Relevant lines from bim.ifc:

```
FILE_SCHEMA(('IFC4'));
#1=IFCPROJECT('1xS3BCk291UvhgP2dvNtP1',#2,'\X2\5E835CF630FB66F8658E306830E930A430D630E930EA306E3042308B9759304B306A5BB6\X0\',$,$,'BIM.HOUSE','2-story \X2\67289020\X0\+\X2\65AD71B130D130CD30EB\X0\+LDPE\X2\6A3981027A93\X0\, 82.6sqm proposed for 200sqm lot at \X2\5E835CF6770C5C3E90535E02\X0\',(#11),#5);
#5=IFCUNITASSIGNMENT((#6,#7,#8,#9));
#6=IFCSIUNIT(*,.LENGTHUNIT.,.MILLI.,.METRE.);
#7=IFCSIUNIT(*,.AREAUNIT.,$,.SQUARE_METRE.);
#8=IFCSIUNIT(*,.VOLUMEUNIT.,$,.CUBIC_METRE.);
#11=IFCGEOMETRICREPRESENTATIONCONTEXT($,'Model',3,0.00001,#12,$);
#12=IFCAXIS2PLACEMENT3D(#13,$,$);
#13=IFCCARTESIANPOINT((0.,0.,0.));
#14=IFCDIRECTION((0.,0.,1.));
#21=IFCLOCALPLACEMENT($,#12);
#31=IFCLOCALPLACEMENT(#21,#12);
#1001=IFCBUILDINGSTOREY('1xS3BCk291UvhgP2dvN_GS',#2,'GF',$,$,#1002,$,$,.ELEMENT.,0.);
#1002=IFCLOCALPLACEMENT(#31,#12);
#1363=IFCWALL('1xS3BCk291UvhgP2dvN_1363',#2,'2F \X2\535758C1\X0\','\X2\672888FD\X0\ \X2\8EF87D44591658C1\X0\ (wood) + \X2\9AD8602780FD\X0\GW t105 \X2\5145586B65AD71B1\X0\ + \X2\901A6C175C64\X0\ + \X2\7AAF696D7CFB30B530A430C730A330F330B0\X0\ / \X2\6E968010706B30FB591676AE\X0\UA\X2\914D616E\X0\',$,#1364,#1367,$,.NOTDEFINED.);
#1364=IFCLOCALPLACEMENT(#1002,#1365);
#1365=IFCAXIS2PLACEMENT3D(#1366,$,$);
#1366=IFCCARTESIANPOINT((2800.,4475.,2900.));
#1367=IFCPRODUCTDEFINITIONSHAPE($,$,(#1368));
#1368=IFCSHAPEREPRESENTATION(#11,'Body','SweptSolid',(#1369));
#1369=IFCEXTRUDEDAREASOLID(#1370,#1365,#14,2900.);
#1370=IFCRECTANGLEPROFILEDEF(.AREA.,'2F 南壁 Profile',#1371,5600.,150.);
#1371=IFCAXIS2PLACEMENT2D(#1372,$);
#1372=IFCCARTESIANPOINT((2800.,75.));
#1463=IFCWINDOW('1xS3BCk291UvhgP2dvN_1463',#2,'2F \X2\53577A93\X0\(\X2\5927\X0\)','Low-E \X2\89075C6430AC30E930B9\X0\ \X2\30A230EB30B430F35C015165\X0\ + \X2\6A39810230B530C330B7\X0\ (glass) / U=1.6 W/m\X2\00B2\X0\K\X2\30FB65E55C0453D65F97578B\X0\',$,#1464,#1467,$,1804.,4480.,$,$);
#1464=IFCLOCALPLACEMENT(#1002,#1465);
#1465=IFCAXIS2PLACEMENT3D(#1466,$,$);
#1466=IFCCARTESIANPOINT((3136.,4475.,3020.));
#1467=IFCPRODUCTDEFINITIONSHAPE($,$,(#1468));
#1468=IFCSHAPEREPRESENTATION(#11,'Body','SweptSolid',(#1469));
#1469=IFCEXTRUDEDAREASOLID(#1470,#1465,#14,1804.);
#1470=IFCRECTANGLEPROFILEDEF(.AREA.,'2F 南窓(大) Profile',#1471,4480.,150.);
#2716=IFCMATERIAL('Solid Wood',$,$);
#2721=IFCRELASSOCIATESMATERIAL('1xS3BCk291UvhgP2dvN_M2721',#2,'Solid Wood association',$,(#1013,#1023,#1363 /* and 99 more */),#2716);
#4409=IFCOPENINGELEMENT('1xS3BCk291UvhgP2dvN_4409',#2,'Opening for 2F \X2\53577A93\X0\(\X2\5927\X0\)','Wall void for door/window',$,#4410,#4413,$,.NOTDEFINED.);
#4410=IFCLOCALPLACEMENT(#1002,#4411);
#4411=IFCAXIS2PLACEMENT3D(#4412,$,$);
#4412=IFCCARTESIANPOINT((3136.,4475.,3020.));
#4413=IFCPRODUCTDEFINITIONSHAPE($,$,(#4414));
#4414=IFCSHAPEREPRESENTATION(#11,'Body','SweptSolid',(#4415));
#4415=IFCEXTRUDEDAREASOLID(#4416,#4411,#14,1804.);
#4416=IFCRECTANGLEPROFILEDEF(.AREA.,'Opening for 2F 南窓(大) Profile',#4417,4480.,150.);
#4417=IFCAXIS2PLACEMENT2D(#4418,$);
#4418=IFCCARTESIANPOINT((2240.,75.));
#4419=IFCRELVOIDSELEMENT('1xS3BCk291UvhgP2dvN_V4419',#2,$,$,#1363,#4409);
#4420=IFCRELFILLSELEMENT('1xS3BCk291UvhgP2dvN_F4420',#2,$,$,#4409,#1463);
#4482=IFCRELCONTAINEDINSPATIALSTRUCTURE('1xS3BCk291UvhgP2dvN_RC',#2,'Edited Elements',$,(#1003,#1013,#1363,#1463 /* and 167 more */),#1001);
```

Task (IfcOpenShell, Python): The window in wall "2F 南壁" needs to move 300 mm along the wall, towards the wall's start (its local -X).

```python
import ifcopenshell
import ifcopenshell.api.geometry
import ifcopenshell.util.placement

model = ifcopenshell.open("bim.ifc")

window = model.by_guid("1xS3BCk291UvhgP2dvN_1463")
opening = window.FillsVoids[0].RelatingOpeningElement
wall = opening.VoidsElements[0].RelatingBuildingElement

wall_matrix = ifcopenshell.util.placement.get_local_placement(wall.ObjectPlacement)
shift = wall_matrix[:3, 0] * -300.0
before = ifcopenshell.util.placement.get_local_placement(window.ObjectPlacement)[:3, 3].copy()

# The window is not placed relative to its opening, so move both.
for product in (opening, window):
    matrix = ifcopenshell.util.placement.get_local_placement(product.ObjectPlacement)
    matrix[:3, 3] += shift
    ifcopenshell.api.geometry.edit_object_placement(model, product=product, matrix=matrix, is_si=False)

after = ifcopenshell.util.placement.get_local_placement(window.ObjectPlacement)[:3, 3]
print("window moved by", (after - before).round(3) + 0.0)

model.write("bim_rev.ifc")
```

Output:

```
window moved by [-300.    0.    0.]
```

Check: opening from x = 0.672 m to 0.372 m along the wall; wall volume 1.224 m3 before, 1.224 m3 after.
